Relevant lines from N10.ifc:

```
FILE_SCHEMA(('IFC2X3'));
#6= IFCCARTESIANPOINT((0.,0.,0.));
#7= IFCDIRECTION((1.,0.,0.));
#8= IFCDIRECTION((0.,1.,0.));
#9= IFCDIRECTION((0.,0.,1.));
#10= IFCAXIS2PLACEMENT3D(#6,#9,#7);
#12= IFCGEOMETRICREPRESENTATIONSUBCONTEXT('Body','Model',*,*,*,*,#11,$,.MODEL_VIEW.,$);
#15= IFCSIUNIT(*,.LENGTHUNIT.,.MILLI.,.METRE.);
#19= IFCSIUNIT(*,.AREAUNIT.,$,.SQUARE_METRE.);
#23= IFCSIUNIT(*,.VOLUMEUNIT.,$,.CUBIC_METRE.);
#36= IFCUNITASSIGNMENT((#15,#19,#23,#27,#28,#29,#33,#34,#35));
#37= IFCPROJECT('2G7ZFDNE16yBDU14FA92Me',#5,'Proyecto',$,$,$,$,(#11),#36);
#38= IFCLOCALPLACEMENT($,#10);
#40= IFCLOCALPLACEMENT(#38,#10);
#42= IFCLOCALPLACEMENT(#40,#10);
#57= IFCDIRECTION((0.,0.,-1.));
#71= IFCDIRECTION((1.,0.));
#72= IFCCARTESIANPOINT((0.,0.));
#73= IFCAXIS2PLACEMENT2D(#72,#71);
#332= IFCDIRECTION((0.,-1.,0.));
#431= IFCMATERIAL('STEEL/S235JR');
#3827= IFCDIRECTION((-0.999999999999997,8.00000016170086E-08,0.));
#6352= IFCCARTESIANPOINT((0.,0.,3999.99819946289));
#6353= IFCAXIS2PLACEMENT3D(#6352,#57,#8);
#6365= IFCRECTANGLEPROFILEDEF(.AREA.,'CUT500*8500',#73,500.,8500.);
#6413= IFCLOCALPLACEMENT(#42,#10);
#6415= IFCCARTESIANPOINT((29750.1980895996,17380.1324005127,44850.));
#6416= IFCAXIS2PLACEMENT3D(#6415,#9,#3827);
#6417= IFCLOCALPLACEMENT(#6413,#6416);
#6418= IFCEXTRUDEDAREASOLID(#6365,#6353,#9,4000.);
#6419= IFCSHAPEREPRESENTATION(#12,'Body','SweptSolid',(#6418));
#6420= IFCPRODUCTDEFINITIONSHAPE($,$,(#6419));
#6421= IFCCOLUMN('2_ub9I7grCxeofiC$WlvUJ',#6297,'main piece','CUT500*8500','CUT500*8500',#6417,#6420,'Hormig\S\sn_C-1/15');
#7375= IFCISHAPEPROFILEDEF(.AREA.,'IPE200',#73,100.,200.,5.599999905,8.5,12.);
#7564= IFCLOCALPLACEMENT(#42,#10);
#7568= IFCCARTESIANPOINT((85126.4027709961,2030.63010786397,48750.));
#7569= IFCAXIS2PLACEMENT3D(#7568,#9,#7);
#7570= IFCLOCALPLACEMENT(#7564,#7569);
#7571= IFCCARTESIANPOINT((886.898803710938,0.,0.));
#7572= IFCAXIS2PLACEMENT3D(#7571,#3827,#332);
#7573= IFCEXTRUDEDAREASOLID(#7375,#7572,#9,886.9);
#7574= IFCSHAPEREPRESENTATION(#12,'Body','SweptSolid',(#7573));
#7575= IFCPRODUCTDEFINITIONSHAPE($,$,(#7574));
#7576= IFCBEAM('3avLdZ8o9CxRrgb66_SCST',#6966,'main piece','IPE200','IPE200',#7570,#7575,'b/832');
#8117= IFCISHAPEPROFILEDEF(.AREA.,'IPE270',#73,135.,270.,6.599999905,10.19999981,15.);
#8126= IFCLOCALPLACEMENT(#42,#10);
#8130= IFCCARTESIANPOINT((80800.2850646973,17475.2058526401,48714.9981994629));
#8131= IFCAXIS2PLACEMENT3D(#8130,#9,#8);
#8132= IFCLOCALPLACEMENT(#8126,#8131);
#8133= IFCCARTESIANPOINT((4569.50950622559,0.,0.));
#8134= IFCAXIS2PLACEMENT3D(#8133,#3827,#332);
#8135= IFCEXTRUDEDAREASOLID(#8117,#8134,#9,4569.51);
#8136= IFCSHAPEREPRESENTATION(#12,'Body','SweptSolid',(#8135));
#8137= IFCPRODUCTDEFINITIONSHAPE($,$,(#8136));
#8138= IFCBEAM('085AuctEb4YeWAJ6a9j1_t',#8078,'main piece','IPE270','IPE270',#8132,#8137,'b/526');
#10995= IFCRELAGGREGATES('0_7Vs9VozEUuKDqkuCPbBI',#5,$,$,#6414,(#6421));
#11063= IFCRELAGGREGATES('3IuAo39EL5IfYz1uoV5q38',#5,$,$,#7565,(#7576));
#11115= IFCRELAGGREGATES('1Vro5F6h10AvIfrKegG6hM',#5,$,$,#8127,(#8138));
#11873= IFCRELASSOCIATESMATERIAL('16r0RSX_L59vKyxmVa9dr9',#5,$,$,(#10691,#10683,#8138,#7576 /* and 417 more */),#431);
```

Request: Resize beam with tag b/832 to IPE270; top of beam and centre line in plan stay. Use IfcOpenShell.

```python
import ifcopenshell
import ifcopenshell.util.element
import ifcopenshell.util.representation

model = ifcopenshell.open("N10.ifc")

member = model.by_id(7576)
source = next(p for p in model.by_type("IfcIShapeProfileDef") if p.ProfileName == "IPE270")

body = ifcopenshell.util.representation.get_representation(member, "Model", "Body")
solid = body.Items[0]
old_profile = solid.SweptArea

# Copy the section's sizes but keep this member's own profile position.
profile = ifcopenshell.util.element.copy(model, source)
# Profiles are centred, so shift by half the change in depth to hold the top.
shift = (old_profile.OverallDepth - profile.OverallDepth) / 2
x, y = old_profile.Position.Location.Coordinates
up = (0.0, 1.0)  # upwards, in the solid's own plane
location = model.createIfcCartesianPoint((x + up[0] * shift, y + up[1] * shift))
profile.Position = model.createIfcAxis2Placement2D(location, old_profile.Position.RefDirection)
solid.SweptArea = profile
if not model.get_total_inverses(old_profile):
    ifcopenshell.util.element.remove_deep2(model, old_profile)
member.Description = member.Description.replace("IPE200", "IPE270")
member.ObjectType = member.ObjectType.replace("IPE200", "IPE270")

print(solid.SweptArea)

model.write("N10_updated.ifc")
```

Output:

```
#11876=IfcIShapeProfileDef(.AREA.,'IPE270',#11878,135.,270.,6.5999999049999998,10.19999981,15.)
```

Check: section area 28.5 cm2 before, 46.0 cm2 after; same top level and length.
